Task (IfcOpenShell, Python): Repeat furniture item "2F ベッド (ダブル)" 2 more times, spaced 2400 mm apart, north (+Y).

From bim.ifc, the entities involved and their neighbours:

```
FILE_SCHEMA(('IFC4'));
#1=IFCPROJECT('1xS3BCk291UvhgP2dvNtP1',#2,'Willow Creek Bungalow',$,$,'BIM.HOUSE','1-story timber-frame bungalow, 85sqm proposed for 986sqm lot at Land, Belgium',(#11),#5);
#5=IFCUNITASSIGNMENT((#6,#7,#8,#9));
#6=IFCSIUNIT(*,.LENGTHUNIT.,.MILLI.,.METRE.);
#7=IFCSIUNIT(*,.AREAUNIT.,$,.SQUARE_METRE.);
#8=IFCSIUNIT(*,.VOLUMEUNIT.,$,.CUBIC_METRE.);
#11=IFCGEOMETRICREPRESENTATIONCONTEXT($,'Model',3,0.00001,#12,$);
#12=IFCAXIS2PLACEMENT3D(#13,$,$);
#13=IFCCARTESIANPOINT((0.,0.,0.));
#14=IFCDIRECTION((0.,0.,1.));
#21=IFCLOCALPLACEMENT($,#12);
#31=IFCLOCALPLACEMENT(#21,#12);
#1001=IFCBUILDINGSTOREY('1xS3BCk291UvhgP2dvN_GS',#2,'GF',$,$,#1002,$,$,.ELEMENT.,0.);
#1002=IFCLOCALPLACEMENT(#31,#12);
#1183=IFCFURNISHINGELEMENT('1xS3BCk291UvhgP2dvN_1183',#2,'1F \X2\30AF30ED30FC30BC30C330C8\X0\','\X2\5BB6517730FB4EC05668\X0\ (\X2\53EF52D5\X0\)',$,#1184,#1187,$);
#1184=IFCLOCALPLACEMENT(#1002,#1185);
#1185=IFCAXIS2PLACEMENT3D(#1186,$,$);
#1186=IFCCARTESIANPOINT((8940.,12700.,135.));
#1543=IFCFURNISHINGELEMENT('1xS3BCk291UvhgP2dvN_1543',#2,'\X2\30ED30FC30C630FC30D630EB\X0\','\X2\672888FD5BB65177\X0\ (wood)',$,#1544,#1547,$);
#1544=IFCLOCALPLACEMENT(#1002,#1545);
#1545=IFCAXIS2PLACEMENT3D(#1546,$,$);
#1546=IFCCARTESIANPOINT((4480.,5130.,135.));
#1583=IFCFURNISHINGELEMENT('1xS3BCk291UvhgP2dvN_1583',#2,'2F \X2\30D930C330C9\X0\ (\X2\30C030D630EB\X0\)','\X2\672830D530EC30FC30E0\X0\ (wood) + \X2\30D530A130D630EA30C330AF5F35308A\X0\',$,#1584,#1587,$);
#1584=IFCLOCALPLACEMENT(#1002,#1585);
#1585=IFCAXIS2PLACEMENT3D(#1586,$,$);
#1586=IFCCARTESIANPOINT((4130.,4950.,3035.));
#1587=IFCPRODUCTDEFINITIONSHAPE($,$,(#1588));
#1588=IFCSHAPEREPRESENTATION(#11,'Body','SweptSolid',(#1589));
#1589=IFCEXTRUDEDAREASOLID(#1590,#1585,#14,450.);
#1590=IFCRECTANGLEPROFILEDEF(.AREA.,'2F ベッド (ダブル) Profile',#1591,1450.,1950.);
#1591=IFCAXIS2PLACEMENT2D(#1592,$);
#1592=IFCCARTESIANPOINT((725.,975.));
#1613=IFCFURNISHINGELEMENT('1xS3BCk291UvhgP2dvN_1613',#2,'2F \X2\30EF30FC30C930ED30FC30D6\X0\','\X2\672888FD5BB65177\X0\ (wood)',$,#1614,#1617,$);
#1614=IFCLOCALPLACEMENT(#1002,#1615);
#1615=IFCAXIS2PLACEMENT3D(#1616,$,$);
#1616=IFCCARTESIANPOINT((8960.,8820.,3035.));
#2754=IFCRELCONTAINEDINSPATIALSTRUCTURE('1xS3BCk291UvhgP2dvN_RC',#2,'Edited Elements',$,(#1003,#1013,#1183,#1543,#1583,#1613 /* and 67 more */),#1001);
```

```python
import numpy as np
import ifcopenshell
import ifcopenshell.api.geometry
import ifcopenshell.api.root
import ifcopenshell.util.element
import ifcopenshell.util.placement
import ifcopenshell.util.unit

model = ifcopenshell.open("bim.ifc")
unit_scale = ifcopenshell.util.unit.calculate_unit_scale(model)


def reuse_history(source, copy):
    """copy_class also copies each property set's owner history, people and application; keep the originals."""
    for rel in copy.IsDefinedBy:
        if rel.is_a("IfcRelDefinesByProperties") and (history := rel.RelatingPropertyDefinition.OwnerHistory):
            rel.RelatingPropertyDefinition.OwnerHistory = source.OwnerHistory
            ifcopenshell.util.element.remove_deep2(model, history)


source = model.by_guid("1xS3BCk291UvhgP2dvN_1583")
base = ifcopenshell.util.placement.get_local_placement(source.ObjectPlacement)
step = np.array([0.0, 1.0, 0.0]) * 2.4 / unit_scale

for i in range(1, 3):
    copy = ifcopenshell.api.root.copy_class(model, product=source)
    copy.Representation = ifcopenshell.util.element.copy_deep(
        model, source.Representation, exclude=["IfcGeometricRepresentationContext", "IfcRepresentationMap"]
    )
    reuse_history(source, copy)
    matrix = base.copy()
    matrix[:3, 3] += i * step
    print("added at", matrix[:3, 3].round(3) + 0.0)
    ifcopenshell.api.geometry.edit_object_placement(model, product=copy, matrix=matrix, is_si=False)

model.write("bim_updated.ifc")
```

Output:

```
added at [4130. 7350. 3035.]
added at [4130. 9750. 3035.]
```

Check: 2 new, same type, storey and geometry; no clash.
